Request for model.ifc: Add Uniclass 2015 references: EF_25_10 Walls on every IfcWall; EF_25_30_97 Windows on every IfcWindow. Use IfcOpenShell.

First a look at what the model holds.

```python
import ifcopenshell

model = ifcopenshell.open("model.ifc")
print(model.schema)
print("classifications:", [c.Name for c in model.by_type("IfcClassification")])
for ifc_class in ("IfcDoor", "IfcRoof", "IfcStair", "IfcWall", "IfcWindow"):
    print(ifc_class, len(model.by_type(ifc_class)))
```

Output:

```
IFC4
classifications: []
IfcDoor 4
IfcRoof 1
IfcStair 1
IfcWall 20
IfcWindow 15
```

```python
import ifcopenshell
import ifcopenshell.api.classification

model = ifcopenshell.open("model.ifc")

system = ifcopenshell.api.classification.add_classification(model, classification="Uniclass 2015")

codes = {
    "IfcWall": ("EF_25_10", "Walls"),
    "IfcWindow": ("EF_25_30_97", "Windows"),
}
for ifc_class, (code, name) in codes.items():
    products = model.by_type(ifc_class)
    ifcopenshell.api.classification.add_reference(
        model, products=products, classification=system, identification=code, name=name
    )
    print(code, len(products))

model.write("model_edited.ifc")
```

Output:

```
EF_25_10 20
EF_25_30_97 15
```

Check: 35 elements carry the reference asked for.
